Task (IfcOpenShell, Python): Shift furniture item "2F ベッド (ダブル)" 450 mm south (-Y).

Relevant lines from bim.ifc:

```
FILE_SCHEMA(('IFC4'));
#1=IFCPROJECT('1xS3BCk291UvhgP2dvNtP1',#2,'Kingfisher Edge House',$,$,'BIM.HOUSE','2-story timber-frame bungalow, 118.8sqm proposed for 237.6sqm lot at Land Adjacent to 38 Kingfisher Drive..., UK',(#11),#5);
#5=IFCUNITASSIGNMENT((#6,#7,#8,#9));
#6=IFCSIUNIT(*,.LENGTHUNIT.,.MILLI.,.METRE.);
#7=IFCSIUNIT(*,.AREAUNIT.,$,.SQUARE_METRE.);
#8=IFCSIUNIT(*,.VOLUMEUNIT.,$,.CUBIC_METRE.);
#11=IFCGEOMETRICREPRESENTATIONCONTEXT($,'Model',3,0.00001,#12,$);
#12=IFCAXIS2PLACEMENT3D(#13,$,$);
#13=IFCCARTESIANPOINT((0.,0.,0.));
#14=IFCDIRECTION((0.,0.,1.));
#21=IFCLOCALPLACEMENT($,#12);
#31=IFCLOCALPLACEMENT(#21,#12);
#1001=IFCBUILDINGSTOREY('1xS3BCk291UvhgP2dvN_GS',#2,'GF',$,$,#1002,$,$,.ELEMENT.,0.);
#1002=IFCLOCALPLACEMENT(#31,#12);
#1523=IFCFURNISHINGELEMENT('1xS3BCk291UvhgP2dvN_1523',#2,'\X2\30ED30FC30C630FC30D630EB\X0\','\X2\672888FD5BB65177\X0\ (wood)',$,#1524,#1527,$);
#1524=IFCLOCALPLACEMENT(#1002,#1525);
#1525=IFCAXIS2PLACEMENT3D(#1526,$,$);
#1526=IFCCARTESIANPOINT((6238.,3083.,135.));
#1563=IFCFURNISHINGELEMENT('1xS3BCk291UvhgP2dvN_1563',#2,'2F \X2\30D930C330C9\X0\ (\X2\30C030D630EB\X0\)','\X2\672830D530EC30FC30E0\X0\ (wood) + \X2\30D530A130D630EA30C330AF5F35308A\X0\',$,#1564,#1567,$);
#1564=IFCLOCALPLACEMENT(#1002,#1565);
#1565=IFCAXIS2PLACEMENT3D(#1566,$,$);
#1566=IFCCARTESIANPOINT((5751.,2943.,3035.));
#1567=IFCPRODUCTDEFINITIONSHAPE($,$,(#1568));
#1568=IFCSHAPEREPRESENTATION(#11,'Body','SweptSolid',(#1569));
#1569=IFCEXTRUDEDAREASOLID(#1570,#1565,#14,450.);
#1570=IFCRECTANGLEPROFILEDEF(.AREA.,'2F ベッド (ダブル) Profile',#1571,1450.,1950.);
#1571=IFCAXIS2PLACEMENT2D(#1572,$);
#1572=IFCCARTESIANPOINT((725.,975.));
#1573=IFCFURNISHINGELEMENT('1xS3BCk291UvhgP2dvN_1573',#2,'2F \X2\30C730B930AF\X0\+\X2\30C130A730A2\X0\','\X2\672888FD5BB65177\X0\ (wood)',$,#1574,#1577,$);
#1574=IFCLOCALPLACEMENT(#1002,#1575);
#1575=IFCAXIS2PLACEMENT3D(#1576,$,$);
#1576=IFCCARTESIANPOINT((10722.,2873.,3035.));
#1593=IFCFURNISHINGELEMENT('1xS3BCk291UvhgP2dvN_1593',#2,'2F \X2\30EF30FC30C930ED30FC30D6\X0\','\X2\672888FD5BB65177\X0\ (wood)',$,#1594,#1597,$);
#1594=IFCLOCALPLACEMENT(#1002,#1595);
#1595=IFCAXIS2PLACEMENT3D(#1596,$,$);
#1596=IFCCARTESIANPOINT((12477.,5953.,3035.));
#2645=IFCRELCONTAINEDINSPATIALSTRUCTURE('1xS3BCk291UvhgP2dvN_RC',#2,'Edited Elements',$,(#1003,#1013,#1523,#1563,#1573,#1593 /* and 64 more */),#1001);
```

```python
import ifcopenshell
import ifcopenshell.api.geometry
import ifcopenshell.util.placement

model = ifcopenshell.open("bim.ifc")

item = model.by_guid("1xS3BCk291UvhgP2dvN_1563")
matrix = ifcopenshell.util.placement.get_local_placement(item.ObjectPlacement)
matrix[1, 3] -= 450.0
ifcopenshell.api.geometry.edit_object_placement(model, product=item, matrix=matrix, is_si=False)

print(ifcopenshell.util.placement.get_local_placement(item.ObjectPlacement).round(3) + 0.0)

model.write("bim_updated.ifc")
```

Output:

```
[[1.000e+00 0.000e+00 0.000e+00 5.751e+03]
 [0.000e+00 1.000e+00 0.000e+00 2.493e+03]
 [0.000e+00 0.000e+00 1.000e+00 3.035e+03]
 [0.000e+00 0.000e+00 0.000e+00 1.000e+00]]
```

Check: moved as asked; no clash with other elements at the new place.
